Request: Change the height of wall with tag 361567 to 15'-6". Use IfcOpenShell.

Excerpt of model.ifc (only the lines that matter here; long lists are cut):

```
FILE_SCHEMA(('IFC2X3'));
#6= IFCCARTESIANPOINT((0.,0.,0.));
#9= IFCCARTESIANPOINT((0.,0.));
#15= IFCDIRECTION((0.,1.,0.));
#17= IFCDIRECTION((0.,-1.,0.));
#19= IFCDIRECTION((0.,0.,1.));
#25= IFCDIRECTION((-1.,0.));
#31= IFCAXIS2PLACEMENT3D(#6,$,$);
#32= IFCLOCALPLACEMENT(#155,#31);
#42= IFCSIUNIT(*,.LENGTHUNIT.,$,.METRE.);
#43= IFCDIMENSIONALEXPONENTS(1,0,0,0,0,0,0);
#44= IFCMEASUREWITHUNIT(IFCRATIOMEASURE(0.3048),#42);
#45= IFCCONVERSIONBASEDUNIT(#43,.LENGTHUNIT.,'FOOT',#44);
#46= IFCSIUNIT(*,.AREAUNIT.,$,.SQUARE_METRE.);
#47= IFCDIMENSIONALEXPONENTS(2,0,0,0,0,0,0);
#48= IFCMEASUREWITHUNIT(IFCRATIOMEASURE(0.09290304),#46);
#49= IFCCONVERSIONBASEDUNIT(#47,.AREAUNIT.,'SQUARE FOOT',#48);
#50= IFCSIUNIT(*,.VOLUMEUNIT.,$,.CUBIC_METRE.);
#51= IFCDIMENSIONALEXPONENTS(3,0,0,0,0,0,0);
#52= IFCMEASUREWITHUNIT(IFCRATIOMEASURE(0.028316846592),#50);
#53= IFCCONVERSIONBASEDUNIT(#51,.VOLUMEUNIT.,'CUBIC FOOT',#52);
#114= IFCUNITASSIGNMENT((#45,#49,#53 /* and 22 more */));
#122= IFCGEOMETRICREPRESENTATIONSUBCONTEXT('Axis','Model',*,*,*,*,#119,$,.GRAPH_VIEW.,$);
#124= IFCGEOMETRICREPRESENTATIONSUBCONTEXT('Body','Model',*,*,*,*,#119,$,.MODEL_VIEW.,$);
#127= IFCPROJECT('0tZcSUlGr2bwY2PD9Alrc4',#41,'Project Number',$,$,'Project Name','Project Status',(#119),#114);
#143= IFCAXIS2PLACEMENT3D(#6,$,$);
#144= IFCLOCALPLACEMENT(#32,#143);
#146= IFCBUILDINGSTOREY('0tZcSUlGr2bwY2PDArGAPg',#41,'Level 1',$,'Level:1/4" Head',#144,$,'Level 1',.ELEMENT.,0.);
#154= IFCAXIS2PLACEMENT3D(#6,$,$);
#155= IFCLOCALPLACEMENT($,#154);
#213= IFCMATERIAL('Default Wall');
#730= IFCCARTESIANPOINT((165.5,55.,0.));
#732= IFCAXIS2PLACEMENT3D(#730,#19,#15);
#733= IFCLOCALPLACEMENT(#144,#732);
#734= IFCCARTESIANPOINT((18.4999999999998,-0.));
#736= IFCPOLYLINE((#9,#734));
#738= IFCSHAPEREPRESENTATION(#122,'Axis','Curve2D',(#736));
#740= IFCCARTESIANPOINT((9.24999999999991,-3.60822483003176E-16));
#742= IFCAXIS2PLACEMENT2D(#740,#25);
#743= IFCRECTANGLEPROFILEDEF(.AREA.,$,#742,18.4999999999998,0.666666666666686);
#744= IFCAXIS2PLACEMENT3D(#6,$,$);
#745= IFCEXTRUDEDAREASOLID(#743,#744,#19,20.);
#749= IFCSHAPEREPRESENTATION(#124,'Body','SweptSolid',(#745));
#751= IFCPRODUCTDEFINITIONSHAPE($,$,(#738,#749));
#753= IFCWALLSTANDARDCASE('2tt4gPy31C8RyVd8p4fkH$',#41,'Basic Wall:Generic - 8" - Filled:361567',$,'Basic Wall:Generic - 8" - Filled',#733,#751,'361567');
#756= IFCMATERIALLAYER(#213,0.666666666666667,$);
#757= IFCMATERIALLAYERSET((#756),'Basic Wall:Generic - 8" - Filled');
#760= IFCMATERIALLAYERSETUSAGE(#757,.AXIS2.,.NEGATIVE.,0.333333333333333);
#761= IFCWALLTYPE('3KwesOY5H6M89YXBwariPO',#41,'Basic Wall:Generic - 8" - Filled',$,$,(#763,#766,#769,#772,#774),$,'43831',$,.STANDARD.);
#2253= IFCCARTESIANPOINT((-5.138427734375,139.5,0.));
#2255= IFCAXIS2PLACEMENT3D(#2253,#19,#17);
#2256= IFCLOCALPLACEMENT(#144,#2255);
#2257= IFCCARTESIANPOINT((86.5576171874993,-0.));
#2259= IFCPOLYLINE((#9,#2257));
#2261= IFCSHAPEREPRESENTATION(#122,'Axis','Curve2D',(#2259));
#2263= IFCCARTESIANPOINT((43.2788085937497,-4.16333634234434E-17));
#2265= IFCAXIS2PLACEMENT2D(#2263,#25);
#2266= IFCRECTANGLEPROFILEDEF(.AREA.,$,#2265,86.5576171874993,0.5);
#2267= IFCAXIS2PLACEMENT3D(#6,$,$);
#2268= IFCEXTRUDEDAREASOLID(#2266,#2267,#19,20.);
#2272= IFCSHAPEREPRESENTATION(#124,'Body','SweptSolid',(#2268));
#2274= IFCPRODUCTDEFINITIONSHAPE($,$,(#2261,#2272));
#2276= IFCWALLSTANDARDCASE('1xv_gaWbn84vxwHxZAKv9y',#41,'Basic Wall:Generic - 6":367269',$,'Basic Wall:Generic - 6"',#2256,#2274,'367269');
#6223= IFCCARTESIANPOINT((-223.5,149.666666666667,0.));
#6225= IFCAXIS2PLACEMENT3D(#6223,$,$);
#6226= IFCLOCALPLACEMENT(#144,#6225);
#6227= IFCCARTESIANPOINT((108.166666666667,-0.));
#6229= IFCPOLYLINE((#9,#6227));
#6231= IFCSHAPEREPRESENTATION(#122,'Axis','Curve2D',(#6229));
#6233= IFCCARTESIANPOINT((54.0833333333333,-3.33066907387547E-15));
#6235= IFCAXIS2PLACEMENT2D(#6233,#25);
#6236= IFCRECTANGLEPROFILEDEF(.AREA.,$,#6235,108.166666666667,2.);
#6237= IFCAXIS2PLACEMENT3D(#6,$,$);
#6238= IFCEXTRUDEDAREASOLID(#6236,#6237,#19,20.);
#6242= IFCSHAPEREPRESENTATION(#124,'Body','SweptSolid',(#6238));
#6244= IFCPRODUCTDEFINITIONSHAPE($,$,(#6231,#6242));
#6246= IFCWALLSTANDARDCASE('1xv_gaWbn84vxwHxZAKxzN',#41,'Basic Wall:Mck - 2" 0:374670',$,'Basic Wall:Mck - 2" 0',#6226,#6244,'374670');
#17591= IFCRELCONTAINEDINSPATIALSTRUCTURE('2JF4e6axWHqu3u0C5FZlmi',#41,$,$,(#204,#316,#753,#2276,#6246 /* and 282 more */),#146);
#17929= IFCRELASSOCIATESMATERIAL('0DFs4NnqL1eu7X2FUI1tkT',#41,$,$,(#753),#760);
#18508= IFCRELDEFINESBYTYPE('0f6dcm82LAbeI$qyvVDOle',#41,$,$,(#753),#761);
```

```python
import ifcopenshell
import ifcopenshell.geom
import ifcopenshell.util.representation
import ifcopenshell.util.shape
import ifcopenshell.util.unit

model = ifcopenshell.open("model.ifc")
unit_scale = ifcopenshell.util.unit.calculate_unit_scale(model)
settings = ifcopenshell.geom.settings()


def volume(element):
    """Net volume in cubic metres, openings subtracted."""
    shape = ifcopenshell.geom.create_shape(settings, element)
    return ifcopenshell.util.shape.get_volume(shape.geometry)


wall = model.by_guid("2tt4gPy31C8RyVd8p4fkH$")
before = volume(wall)

body = ifcopenshell.util.representation.get_representation(wall, "Model", "Body")
solid = body.Items[0]
old_height = solid.Depth
solid.Depth = 186 * 0.0254 / unit_scale
after = volume(wall)

print(f"height {old_height:g} -> {solid.Depth:g}, volume {before:.3f} -> {after:.3f} m3")

model.write("model-out.ifc")
```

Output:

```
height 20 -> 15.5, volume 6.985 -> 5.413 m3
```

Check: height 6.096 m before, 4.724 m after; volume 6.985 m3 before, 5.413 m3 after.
